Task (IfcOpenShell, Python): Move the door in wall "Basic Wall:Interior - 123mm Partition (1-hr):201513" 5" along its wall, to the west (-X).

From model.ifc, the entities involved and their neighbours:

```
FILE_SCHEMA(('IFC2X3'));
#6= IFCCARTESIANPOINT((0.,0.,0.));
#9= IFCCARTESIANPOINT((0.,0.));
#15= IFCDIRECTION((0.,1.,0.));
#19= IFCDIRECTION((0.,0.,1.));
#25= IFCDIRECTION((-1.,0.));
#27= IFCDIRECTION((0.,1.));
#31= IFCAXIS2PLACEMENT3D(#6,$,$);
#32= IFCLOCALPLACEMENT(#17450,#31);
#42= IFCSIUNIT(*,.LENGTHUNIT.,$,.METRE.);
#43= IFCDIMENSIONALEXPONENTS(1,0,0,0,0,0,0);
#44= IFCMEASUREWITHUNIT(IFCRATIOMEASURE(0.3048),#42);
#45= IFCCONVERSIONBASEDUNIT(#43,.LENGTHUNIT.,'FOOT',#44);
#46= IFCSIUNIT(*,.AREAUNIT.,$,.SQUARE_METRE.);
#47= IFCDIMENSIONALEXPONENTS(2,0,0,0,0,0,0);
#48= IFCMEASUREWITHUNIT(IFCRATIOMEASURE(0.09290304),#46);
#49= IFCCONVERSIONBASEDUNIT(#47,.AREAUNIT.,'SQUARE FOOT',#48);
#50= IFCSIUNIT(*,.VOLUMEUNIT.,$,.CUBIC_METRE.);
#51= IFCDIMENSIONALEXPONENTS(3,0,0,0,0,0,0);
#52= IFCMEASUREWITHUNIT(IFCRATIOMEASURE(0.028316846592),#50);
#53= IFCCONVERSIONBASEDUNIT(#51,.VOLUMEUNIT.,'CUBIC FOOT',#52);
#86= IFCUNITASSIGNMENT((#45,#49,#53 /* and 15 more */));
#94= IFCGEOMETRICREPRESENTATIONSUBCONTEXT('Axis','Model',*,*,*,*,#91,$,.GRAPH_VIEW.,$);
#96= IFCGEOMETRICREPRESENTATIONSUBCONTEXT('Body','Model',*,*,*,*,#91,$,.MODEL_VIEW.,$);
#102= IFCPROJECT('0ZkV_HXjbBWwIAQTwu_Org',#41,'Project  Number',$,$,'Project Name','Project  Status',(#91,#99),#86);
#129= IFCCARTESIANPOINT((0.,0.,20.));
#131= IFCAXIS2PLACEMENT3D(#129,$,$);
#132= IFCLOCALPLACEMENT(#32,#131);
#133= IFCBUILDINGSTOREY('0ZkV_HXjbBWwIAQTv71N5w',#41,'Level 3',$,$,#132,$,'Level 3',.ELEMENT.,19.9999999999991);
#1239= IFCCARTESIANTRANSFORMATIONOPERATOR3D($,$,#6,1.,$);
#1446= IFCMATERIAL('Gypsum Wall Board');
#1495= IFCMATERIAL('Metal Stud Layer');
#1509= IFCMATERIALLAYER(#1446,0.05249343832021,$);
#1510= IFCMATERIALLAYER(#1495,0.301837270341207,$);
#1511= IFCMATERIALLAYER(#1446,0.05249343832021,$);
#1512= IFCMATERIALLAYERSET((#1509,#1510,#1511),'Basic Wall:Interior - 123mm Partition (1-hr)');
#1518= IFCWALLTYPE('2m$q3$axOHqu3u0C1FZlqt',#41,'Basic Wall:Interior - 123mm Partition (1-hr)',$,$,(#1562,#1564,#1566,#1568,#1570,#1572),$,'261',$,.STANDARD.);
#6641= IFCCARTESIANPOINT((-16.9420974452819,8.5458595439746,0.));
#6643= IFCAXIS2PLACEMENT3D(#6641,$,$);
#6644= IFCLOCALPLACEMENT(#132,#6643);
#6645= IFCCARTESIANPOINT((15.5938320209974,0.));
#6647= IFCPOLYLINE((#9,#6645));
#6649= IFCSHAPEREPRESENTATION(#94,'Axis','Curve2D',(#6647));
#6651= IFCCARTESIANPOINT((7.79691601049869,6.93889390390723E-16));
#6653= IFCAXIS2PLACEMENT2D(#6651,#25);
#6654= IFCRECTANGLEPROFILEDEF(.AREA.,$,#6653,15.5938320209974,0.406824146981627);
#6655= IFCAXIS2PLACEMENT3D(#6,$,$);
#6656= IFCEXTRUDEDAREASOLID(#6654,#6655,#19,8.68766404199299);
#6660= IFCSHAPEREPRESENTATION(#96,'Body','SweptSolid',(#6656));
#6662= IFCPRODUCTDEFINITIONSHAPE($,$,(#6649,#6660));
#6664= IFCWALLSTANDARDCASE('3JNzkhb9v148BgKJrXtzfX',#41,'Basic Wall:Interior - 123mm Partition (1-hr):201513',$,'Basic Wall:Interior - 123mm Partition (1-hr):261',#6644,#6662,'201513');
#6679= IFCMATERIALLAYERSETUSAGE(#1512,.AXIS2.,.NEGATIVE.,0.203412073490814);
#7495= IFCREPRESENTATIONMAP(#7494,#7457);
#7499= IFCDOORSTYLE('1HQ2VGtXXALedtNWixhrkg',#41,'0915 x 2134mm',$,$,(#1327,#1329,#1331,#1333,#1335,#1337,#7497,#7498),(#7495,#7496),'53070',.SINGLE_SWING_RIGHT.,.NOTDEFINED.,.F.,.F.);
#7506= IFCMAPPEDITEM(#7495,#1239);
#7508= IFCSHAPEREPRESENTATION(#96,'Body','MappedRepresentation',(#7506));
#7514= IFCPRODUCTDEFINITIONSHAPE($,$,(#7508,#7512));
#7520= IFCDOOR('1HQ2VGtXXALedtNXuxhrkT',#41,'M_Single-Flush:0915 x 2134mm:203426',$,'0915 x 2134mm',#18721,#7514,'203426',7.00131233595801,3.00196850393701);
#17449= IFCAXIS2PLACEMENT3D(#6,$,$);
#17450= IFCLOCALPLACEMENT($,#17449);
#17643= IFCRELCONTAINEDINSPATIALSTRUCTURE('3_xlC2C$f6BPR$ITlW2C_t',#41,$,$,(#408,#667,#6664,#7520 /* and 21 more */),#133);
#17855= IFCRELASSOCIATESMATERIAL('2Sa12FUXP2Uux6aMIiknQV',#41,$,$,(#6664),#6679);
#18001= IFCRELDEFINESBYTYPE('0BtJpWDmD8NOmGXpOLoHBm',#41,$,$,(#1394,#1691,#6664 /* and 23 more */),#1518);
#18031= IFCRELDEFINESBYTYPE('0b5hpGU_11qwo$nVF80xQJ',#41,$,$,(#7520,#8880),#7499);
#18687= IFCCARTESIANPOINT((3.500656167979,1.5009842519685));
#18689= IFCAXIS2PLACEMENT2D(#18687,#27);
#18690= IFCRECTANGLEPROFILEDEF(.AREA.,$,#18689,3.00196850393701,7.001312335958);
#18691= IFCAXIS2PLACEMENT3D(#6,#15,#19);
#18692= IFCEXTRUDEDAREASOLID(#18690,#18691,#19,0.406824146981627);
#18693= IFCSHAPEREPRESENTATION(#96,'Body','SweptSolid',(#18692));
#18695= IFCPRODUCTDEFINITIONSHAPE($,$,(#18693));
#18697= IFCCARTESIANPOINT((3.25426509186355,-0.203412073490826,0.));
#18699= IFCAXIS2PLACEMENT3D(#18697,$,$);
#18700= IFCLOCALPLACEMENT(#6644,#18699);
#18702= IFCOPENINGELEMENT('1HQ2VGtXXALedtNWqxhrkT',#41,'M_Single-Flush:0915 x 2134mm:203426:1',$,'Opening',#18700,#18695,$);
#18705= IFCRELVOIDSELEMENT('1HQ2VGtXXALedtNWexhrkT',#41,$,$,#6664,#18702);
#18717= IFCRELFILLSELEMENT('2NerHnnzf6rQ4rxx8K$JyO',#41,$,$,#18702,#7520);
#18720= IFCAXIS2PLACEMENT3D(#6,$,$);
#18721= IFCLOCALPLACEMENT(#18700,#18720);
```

```python
import ifcopenshell
import ifcopenshell.api.geometry
import ifcopenshell.util.placement
import ifcopenshell.util.unit

model = ifcopenshell.open("model.ifc")
unit_scale = ifcopenshell.util.unit.calculate_unit_scale(model)

door = model.by_guid("1HQ2VGtXXALedtNXuxhrkT")
opening = door.FillsVoids[0].RelatingOpeningElement
wall = opening.VoidsElements[0].RelatingBuildingElement

wall_matrix = ifcopenshell.util.placement.get_local_placement(wall.ObjectPlacement)
shift = wall_matrix[:3, 0] * -5 * 0.0254 / unit_scale
before = ifcopenshell.util.placement.get_local_placement(door.ObjectPlacement)[:3, 3].copy()

# The door is placed relative to its opening, so it follows when the opening moves.
matrix = ifcopenshell.util.placement.get_local_placement(opening.ObjectPlacement)
matrix[:3, 3] += shift
ifcopenshell.api.geometry.edit_object_placement(
    model, product=opening, matrix=matrix, is_si=False, should_transform_children=True
)

after = ifcopenshell.util.placement.get_local_placement(door.ObjectPlacement)[:3, 3]
print("door moved by", (after - before).round(3) + 0.0)

model.write("model_edited.ifc")
```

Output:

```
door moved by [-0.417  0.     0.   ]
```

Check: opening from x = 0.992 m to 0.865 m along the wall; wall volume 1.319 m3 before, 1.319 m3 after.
